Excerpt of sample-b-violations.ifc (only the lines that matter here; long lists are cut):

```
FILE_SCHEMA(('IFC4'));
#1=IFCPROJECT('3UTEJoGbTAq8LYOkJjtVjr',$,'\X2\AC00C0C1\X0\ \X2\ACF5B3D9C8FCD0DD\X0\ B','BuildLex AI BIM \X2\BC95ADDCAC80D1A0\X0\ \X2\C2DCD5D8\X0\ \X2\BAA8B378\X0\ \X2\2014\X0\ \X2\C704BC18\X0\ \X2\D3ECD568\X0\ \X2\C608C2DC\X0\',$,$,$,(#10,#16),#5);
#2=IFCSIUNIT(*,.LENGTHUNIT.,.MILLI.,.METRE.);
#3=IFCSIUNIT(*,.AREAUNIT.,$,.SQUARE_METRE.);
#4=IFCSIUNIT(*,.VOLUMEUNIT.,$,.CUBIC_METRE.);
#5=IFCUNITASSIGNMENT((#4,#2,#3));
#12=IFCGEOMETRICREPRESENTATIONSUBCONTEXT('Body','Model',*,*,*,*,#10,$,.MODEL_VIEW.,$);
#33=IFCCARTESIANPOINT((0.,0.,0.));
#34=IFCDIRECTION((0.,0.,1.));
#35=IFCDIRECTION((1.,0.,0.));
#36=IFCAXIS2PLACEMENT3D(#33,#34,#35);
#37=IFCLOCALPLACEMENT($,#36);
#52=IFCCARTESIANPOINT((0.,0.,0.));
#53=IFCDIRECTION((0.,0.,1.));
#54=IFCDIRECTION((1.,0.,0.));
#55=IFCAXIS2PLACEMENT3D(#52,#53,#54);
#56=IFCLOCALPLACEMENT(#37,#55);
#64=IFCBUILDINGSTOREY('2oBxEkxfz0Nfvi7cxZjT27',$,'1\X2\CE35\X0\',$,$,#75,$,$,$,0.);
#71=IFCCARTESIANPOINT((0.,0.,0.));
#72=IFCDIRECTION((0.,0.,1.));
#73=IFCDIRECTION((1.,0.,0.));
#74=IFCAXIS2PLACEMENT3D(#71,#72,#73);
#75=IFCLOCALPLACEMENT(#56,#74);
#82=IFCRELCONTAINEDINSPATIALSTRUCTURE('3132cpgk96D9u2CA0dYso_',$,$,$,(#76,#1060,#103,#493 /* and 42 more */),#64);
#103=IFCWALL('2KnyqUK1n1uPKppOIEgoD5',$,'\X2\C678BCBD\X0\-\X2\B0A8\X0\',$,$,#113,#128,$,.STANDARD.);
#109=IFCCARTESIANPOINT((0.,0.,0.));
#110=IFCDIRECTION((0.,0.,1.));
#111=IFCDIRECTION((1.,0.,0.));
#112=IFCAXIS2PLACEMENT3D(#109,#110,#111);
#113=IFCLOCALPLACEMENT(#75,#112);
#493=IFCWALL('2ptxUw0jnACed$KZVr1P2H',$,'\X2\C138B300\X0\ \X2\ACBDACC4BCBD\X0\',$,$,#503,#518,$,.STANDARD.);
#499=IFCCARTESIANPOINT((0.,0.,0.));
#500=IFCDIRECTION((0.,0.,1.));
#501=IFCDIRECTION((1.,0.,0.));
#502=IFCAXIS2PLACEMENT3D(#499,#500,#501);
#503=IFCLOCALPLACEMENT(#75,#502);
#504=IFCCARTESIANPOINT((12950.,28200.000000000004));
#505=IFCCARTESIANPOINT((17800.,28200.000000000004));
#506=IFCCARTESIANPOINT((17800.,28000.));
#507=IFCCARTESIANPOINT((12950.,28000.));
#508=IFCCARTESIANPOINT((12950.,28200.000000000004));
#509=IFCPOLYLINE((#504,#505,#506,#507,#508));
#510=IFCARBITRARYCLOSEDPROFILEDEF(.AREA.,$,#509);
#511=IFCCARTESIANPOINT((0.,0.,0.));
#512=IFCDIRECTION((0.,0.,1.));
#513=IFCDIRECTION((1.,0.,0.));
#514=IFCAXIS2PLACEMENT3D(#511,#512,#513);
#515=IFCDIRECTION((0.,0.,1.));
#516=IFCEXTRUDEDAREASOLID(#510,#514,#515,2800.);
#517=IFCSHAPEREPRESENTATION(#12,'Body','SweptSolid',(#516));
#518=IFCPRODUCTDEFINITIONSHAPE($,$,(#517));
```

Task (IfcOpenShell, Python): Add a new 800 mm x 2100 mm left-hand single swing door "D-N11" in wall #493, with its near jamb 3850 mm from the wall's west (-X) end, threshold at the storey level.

```python
import numpy as np
import ifcopenshell
import ifcopenshell.api.feature
import ifcopenshell.api.geometry
import ifcopenshell.api.root
import ifcopenshell.api.spatial
import ifcopenshell.geom
import ifcopenshell.util.element
import ifcopenshell.util.placement
import ifcopenshell.util.representation
import ifcopenshell.util.shape
import ifcopenshell.util.unit

model = ifcopenshell.open("sample-b-violations.ifc")
unit_scale = ifcopenshell.util.unit.calculate_unit_scale(model)
settings = ifcopenshell.geom.settings()


def volume(element):
    """Net volume in cubic metres, openings subtracted."""
    shape = ifcopenshell.geom.create_shape(settings, element)
    return ifcopenshell.util.shape.get_volume(shape.geometry)


wall = model.by_id(493)
storey = ifcopenshell.util.element.get_container(wall, ifc_class="IfcBuildingStorey")
context = ifcopenshell.util.representation.get_context(model, "Model", "Body", "MODEL_VIEW")
before = volume(wall)

width, height, from_end, sill = 0.8, 2.1, 3.85, 0.0  # metres

# The wall runs along its own X axis, and the end named is its -X end.
wall_shape = ifcopenshell.geom.create_shape(settings, wall)
x, y, z = ifcopenshell.util.shape.get_vertices(wall_shape.geometry).T
start = x.min() + from_end
face, thickness = float(y.min()), float(y.max() - y.min())
wall_matrix = ifcopenshell.util.placement.get_local_placement(wall.ObjectPlacement)
level = ifcopenshell.util.placement.get_local_placement(storey.ObjectPlacement)[2, 3]


def in_wall(x, y):
    """Placement at x, y metres in the wall's axes, at sill height."""
    matrix = wall_matrix.copy()
    matrix[:, 3] = wall_matrix @ np.array([x / unit_scale, y / unit_scale, 0.0, 1.0])
    matrix[2, 3] = level + sill / unit_scale
    return matrix


# Opening: a box that overshoots both wall faces by 50 mm.
opening = ifcopenshell.api.root.create_entity(model, ifc_class="IfcOpeningElement", predefined_type="OPENING")
box = ifcopenshell.api.geometry.add_wall_representation(
    model, context=context, length=width, height=height, thickness=thickness + 0.1
)
ifcopenshell.api.geometry.assign_representation(model, product=opening, representation=box)
ifcopenshell.api.geometry.edit_object_placement(model, product=opening, matrix=in_wall(start, face - 0.05), is_si=False)
ifcopenshell.api.feature.add_feature(model, feature=opening, element=wall)

door = ifcopenshell.api.root.create_entity(model, ifc_class="IfcDoor", name="D-N11", predefined_type="DOOR")
door.OverallWidth, door.OverallHeight = width / unit_scale, height / unit_scale
door.OperationType = "SINGLE_SWING_LEFT"
body = ifcopenshell.api.geometry.add_door_representation(
    model,
    context=context,
    overall_width=door.OverallWidth,
    overall_height=door.OverallHeight,
    operation_type="SINGLE_SWING_LEFT",
    lining_properties={"LiningDepth": thickness / unit_scale, "ThresholdDepth": thickness / unit_scale},
)
ifcopenshell.api.geometry.assign_representation(model, product=door, representation=body)
ifcopenshell.api.spatial.assign_container(model, products=[door], relating_structure=storey)
ifcopenshell.api.feature.add_filling(model, opening=opening, element=door)

# The lining spans the wall, so the door starts at the wall face.
ifcopenshell.api.geometry.edit_object_placement(model, product=door, matrix=in_wall(start, face), is_si=False)

after = volume(wall)

print(f"wall volume {before:.3f} -> {after:.3f} m3")

model.write("sample-b-violations_rev.ifc")
```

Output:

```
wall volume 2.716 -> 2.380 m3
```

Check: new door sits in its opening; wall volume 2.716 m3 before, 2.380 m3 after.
